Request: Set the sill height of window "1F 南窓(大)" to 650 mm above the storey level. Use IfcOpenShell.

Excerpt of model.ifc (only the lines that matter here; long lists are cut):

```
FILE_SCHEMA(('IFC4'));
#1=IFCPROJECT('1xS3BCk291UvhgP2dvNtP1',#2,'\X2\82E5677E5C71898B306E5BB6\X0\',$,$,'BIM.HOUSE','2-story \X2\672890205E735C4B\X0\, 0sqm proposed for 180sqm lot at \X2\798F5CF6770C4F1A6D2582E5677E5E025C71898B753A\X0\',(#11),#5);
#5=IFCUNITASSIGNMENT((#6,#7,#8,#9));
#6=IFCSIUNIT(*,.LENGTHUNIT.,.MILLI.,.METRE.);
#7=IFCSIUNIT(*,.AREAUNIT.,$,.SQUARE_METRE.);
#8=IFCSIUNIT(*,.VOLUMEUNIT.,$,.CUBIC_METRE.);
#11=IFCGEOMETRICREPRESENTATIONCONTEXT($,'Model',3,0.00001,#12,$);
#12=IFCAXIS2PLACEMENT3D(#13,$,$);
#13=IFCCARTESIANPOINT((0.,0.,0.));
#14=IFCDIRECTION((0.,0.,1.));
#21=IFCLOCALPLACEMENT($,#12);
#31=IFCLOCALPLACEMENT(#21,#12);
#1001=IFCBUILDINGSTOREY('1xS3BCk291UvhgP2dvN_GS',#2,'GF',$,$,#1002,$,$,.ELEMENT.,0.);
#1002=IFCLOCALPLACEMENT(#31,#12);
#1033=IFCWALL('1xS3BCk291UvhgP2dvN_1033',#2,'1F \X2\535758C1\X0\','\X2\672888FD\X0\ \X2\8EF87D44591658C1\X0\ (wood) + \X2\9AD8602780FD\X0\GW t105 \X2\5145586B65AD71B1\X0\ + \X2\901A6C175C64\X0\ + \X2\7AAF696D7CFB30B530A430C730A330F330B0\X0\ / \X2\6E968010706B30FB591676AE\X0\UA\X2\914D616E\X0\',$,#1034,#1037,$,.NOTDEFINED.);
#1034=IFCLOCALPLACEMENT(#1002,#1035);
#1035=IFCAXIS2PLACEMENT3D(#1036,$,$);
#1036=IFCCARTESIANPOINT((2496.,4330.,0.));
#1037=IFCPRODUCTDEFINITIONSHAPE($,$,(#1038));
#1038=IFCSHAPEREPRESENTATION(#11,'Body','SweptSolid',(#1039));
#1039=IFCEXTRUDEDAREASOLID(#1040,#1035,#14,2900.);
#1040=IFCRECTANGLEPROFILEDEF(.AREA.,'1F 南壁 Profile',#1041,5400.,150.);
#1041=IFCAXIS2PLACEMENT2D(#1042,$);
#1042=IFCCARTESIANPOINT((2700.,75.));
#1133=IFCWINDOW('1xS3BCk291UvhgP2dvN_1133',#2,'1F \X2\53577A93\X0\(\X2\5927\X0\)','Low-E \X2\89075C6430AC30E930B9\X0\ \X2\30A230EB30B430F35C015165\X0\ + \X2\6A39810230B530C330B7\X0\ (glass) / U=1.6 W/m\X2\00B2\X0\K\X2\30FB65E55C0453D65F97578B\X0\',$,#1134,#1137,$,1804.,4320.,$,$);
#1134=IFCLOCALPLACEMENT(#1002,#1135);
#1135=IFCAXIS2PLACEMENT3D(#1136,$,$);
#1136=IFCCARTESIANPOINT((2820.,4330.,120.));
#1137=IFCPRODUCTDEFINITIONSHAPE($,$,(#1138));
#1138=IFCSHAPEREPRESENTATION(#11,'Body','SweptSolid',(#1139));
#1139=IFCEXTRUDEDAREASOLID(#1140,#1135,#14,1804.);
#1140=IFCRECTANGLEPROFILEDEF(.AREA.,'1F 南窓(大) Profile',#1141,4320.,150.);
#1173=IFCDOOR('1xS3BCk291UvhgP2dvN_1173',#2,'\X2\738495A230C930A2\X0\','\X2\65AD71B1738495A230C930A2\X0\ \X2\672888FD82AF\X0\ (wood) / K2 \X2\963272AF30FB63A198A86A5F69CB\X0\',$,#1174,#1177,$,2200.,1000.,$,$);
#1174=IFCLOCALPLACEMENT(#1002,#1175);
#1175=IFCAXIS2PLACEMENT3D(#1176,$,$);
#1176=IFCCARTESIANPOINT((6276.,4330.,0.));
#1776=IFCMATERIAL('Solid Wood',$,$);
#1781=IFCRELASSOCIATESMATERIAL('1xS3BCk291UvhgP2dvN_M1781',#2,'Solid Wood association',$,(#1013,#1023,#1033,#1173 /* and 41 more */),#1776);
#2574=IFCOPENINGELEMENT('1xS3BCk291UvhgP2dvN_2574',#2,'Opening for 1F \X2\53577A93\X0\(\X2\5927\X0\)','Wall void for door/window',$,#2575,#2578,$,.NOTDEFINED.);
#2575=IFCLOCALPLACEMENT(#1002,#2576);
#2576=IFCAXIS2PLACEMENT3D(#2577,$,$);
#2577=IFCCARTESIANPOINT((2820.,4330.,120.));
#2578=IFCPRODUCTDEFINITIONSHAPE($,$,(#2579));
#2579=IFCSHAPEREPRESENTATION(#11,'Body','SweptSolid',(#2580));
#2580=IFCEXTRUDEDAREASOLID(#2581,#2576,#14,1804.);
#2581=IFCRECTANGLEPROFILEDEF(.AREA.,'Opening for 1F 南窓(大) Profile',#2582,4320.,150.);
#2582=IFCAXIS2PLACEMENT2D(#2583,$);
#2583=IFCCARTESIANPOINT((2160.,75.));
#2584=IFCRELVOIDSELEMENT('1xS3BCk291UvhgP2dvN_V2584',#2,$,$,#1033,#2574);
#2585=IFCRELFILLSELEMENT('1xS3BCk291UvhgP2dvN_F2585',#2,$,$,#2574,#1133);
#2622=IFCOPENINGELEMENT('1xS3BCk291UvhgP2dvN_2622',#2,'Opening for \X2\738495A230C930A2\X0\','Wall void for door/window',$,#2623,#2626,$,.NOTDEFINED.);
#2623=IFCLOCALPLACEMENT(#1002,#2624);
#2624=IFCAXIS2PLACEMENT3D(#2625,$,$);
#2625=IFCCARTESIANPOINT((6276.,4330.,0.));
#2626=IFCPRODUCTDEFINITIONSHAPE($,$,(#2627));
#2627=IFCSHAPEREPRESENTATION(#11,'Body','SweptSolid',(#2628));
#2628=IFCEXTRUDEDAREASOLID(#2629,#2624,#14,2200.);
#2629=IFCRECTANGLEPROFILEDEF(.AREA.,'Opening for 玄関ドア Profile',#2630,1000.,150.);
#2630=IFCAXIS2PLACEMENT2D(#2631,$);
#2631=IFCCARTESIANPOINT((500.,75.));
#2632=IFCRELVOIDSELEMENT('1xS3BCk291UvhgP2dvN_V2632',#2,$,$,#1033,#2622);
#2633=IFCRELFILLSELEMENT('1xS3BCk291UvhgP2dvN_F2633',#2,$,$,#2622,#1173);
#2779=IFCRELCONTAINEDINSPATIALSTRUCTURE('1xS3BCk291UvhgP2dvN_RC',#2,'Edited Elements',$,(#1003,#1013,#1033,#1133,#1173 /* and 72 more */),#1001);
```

```python
import numpy as np
import ifcopenshell
import ifcopenshell.api.geometry
import ifcopenshell.geom
import ifcopenshell.util.element
import ifcopenshell.util.placement
import ifcopenshell.util.shape
import ifcopenshell.util.unit

model = ifcopenshell.open("model.ifc")
unit_scale = ifcopenshell.util.unit.calculate_unit_scale(model)

window = model.by_guid("1xS3BCk291UvhgP2dvN_1133")
opening = window.FillsVoids[0].RelatingOpeningElement
storey = ifcopenshell.util.element.get_container(window, ifc_class="IfcBuildingStorey")
level = ifcopenshell.util.placement.get_local_placement(storey.ObjectPlacement)[2, 3]

# The opening's origin need not be at the sill, so measure its lowest point.
shape = ifcopenshell.geom.create_shape(ifcopenshell.geom.settings(), opening)
bottom = ifcopenshell.util.shape.get_shape_bottom_elevation(shape, shape.geometry) / unit_scale
dz = level + 0.65 / unit_scale - bottom

shift = np.array([0.0, 0.0, dz])
# The window is not placed relative to its opening, so move both.
for product in (opening, window):
    matrix = ifcopenshell.util.placement.get_local_placement(product.ObjectPlacement)
    matrix[:3, 3] += shift
    ifcopenshell.api.geometry.edit_object_placement(model, product=product, matrix=matrix, is_si=False)

print(f"moved by {dz * unit_scale:+.3f} m")

model.write("model_updated.ifc")
```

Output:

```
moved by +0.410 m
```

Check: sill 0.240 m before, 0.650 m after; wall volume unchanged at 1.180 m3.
